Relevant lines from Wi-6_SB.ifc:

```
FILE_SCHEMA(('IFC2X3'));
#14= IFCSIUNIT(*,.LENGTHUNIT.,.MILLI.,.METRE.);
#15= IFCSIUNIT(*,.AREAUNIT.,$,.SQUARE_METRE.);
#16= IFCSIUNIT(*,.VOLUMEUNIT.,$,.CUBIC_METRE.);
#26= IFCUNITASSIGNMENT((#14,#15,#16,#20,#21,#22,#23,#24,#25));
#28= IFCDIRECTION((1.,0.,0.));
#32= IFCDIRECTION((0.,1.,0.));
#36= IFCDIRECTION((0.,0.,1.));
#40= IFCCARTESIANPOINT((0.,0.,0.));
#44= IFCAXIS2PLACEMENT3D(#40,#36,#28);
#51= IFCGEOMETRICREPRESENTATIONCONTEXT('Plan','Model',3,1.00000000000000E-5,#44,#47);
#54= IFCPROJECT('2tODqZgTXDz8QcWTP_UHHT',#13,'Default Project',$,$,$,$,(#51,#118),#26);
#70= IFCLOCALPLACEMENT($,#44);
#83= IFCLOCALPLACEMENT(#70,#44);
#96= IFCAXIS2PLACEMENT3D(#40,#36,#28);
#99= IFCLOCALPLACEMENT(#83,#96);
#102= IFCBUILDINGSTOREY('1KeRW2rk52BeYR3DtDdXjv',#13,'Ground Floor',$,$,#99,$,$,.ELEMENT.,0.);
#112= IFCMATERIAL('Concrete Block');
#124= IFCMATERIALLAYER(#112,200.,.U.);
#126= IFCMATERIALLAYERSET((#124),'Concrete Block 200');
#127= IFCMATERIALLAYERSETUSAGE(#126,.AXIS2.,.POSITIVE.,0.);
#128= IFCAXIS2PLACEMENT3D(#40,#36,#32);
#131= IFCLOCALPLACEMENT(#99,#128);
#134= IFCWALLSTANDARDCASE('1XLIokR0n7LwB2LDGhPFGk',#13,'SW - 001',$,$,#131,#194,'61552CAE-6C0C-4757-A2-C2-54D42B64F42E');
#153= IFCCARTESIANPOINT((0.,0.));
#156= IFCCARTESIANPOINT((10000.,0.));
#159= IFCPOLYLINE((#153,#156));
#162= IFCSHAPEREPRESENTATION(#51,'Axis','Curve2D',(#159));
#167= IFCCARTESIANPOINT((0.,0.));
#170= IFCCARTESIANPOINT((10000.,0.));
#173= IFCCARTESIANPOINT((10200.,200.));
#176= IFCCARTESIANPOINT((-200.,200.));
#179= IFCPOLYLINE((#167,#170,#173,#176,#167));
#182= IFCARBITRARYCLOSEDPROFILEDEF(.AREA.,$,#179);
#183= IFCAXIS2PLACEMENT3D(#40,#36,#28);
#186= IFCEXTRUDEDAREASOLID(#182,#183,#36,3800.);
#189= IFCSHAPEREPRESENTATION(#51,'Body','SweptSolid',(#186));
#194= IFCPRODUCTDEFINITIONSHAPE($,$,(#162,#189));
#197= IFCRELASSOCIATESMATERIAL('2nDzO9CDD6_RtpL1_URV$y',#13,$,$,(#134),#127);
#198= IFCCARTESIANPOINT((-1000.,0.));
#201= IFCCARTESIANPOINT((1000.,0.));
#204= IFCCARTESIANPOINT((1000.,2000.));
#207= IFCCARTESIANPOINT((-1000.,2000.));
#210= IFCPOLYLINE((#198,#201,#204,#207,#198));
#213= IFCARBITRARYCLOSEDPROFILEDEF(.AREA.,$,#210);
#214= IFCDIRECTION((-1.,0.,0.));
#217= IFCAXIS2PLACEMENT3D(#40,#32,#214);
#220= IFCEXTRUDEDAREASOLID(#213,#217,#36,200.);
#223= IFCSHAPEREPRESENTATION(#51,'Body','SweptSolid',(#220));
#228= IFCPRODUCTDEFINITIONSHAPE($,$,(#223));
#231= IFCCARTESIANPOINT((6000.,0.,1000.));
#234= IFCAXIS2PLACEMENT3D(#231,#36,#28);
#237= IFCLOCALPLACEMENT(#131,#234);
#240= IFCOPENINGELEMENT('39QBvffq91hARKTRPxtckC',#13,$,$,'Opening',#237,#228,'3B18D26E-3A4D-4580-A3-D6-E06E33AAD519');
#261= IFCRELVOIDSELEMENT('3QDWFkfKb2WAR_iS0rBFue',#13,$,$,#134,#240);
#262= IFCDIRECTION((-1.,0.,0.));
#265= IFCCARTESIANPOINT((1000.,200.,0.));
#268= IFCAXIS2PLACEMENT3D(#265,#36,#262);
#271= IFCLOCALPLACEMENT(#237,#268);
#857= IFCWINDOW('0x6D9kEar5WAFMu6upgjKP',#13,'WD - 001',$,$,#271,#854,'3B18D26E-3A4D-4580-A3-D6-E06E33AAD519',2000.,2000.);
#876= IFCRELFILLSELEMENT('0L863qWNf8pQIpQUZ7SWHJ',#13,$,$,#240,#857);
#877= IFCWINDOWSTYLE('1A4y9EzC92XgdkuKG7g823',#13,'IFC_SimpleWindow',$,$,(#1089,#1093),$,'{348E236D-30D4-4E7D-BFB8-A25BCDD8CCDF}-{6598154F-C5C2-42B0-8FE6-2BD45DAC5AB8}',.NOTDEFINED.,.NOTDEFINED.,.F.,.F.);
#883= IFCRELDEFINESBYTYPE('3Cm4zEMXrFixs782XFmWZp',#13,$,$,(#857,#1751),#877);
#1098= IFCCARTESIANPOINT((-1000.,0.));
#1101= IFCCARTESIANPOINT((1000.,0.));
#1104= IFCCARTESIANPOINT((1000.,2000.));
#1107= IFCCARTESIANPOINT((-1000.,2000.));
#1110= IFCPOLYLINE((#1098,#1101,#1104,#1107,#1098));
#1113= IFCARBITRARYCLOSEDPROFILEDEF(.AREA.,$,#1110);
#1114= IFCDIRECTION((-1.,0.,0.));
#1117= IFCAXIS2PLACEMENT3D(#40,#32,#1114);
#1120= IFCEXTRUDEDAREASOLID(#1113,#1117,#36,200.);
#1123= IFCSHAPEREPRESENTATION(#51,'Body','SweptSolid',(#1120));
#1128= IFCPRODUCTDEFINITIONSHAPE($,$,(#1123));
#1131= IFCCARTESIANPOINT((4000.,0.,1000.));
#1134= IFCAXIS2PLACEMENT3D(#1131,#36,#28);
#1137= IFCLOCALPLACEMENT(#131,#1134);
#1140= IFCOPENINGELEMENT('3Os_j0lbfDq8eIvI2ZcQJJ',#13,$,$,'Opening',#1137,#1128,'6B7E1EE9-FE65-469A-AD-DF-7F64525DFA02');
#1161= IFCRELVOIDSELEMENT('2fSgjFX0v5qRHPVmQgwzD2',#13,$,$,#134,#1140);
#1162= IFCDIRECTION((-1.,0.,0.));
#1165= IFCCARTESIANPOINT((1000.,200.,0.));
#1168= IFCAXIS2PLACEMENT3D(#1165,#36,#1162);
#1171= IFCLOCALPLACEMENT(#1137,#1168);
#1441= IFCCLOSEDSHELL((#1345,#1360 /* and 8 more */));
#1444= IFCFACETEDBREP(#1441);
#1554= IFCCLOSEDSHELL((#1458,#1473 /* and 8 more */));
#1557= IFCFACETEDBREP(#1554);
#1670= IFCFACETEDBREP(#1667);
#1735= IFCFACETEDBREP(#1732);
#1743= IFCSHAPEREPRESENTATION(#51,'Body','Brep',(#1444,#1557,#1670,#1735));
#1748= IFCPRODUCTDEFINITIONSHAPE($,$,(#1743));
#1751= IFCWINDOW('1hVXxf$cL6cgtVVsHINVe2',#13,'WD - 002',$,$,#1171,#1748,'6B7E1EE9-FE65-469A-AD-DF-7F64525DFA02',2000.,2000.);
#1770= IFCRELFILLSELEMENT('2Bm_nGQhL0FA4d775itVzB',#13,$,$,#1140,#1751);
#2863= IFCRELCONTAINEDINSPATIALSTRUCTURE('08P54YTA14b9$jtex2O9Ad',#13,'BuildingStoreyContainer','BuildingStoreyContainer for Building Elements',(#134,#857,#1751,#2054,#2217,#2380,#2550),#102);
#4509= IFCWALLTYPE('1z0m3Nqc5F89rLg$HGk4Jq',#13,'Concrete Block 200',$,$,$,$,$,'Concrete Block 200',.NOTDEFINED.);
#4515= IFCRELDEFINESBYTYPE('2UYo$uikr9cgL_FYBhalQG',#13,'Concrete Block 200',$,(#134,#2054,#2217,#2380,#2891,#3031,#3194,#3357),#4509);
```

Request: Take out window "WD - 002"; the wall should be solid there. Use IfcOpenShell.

```python
import ifcopenshell
import ifcopenshell.api.feature
import ifcopenshell.api.root
import ifcopenshell.geom
import ifcopenshell.util.shape

model = ifcopenshell.open("Wi-6_SB.ifc")
settings = ifcopenshell.geom.settings()


def volume(element):
    """Net volume in cubic metres, openings subtracted."""
    shape = ifcopenshell.geom.create_shape(settings, element)
    return ifcopenshell.util.shape.get_volume(shape.geometry)


window = model.by_guid("1hVXxf$cL6cgtVVsHINVe2")
opening = window.FillsVoids[0].RelatingOpeningElement
wall = opening.VoidsElements[0].RelatingBuildingElement
before = volume(wall)

ifcopenshell.api.root.remove_product(model, product=window)
ifcopenshell.api.feature.remove_feature(model, feature=opening)

after = volume(wall)

print(f"wall volume {before:.3f} -> {after:.3f} m3")

model.write("Wi-6_SB_updated.ifc")
```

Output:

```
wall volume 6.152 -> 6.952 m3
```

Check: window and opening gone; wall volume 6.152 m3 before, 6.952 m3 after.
